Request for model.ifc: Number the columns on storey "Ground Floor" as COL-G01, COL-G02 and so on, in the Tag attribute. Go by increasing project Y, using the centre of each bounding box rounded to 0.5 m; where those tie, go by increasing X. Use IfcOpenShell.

First a look at what the model holds.

```python
import ifcopenshell
import ifcopenshell.util.element
import ifcopenshell.util.placement

model = ifcopenshell.open("model.ifc")
print(model.schema)
storey = next(s for s in model.by_type("IfcBuildingStorey") if s.Name == "Ground Floor")
columns = [e for e in ifcopenshell.util.element.get_decomposition(storey) if e.is_a("IfcColumn")]
for e in sorted(columns, key=lambda e: e.id()):
    origin = ifcopenshell.util.placement.get_local_placement(e.ObjectPlacement)[:3, 3]
    print(e.id(), e.Tag, e.Name, origin.round(2) + 0.0, sep=" | ")
```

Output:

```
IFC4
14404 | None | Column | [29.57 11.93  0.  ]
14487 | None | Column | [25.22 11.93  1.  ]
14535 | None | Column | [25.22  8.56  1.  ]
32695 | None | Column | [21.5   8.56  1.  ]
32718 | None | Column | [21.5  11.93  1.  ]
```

```python
import ifcopenshell
import ifcopenshell.geom
import ifcopenshell.util.element
import ifcopenshell.util.shape

model = ifcopenshell.open("model.ifc")
settings = ifcopenshell.geom.settings()
settings.set("use-world-coords", True)


def centre(element):
    shape = ifcopenshell.geom.create_shape(settings, element)
    return ifcopenshell.util.shape.get_bbox_centroid(shape.geometry)


storey = next(s for s in model.by_type("IfcBuildingStorey") if s.Name == "Ground Floor")
columns = [e for e in ifcopenshell.util.element.get_decomposition(storey) if e.is_a("IfcColumn")]

# Insertion points can sit at a corner or the storey origin, so sort by the geometry (in metres).
centres = {e: centre(e) for e in columns}
columns.sort(key=lambda e: (round(centres[e][1] / 0.5), centres[e][0]))

for i, e in enumerate(columns, start=1):
    number = f"COL-G{i:02d}"
    e.Tag = number
    print(e.id(), number)

model.write("model-out.ifc")
```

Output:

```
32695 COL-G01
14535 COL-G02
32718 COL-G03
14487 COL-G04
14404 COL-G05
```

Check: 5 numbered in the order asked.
